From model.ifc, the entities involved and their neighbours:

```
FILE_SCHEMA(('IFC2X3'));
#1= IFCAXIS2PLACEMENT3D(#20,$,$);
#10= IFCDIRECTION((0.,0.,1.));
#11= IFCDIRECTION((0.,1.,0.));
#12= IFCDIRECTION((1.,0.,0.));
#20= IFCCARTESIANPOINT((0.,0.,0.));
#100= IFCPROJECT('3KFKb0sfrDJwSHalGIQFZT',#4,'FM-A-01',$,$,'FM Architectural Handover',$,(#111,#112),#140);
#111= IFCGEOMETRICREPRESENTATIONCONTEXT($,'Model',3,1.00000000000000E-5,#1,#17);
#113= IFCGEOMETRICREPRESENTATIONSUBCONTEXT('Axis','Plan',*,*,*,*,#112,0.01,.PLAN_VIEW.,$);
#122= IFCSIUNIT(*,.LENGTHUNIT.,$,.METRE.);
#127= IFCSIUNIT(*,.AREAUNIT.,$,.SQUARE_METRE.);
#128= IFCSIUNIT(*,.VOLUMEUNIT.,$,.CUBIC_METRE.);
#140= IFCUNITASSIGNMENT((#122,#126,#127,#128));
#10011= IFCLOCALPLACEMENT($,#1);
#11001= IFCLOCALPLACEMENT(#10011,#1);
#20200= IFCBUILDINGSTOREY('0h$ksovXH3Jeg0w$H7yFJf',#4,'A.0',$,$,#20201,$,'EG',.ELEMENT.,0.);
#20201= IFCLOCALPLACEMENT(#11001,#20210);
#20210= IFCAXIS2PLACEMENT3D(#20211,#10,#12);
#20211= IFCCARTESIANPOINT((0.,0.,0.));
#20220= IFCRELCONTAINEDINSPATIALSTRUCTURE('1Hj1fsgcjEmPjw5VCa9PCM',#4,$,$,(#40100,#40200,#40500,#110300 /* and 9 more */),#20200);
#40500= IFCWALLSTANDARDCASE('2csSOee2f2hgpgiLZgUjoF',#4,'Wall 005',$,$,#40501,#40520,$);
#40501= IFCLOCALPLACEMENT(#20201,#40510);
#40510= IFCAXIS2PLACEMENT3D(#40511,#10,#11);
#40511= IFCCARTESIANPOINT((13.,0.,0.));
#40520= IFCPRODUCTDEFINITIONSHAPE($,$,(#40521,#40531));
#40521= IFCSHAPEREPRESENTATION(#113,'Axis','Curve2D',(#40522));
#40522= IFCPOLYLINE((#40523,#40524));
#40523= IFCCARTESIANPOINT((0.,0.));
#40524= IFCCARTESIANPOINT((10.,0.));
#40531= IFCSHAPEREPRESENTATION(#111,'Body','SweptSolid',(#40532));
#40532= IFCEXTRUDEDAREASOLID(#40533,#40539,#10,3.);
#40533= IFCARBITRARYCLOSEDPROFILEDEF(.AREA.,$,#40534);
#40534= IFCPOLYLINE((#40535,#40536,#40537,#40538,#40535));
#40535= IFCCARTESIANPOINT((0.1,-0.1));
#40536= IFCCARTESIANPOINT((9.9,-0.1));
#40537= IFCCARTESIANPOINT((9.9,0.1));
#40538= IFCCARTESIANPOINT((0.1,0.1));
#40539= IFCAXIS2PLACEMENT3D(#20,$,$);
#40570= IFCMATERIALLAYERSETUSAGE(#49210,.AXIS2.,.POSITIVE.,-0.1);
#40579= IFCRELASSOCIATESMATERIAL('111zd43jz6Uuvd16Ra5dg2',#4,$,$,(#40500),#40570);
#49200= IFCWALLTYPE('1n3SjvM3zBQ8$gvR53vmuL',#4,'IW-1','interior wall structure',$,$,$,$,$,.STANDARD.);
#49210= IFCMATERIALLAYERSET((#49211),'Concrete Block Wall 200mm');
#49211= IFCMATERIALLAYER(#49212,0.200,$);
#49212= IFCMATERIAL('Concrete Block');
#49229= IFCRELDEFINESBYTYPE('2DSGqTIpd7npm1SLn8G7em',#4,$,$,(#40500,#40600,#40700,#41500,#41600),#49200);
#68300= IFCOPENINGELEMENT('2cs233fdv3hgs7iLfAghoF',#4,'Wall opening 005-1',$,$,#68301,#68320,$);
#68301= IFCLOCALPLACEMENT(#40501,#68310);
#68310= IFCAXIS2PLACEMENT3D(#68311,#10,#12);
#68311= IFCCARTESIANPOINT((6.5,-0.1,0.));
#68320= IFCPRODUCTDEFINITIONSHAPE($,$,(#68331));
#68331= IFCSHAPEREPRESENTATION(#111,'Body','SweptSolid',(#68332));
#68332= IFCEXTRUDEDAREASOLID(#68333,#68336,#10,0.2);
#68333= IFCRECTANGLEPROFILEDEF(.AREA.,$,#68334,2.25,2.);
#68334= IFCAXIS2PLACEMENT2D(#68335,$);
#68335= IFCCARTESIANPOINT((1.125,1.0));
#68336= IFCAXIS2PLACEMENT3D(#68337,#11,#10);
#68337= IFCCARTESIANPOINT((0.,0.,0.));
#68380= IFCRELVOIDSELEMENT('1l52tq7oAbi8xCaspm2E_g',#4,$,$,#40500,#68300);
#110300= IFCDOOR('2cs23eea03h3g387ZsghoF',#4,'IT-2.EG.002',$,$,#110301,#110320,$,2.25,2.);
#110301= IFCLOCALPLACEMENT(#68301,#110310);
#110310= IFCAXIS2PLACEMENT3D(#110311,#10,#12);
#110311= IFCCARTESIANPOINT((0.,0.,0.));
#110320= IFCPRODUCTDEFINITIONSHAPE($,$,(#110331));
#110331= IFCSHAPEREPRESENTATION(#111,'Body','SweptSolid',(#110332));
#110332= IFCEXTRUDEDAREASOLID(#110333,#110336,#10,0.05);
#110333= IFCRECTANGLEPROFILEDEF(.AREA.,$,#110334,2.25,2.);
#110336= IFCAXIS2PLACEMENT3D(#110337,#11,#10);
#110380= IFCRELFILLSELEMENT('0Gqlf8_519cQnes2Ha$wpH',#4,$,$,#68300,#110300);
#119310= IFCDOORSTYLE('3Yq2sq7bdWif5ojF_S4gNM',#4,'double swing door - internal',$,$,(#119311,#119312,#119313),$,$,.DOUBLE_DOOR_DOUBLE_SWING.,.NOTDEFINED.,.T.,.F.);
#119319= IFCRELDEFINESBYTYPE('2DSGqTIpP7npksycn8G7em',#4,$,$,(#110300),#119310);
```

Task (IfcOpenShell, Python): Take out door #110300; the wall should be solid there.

```python
import ifcopenshell
import ifcopenshell.api.feature
import ifcopenshell.api.root
import ifcopenshell.geom
import ifcopenshell.util.shape

model = ifcopenshell.open("model.ifc")
settings = ifcopenshell.geom.settings()


def volume(element):
    """Net volume in cubic metres, openings subtracted."""
    shape = ifcopenshell.geom.create_shape(settings, element)
    return ifcopenshell.util.shape.get_volume(shape.geometry)


door = model.by_guid("2cs23eea03h3g387ZsghoF")
opening = door.FillsVoids[0].RelatingOpeningElement
wall = opening.VoidsElements[0].RelatingBuildingElement
before = volume(wall)

ifcopenshell.api.root.remove_product(model, product=door)
ifcopenshell.api.feature.remove_feature(model, feature=opening)

after = volume(wall)

print(f"wall volume {before:.3f} -> {after:.3f} m3")

model.write("model_updated.ifc")
```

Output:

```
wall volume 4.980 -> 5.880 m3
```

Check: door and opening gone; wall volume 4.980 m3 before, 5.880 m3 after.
